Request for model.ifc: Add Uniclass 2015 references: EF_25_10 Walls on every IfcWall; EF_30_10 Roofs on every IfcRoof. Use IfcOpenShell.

First a look at what the model holds.

```python
import ifcopenshell

model = ifcopenshell.open("model.ifc")
print(model.schema)
print("classifications:", [c.Name for c in model.by_type("IfcClassification")])
for ifc_class in ("IfcDoor", "IfcRoof", "IfcStair", "IfcWall", "IfcWindow"):
    print(ifc_class, len(model.by_type(ifc_class)))
```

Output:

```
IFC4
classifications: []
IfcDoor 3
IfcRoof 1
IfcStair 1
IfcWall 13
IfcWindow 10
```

```python
import ifcopenshell
import ifcopenshell.api.classification

model = ifcopenshell.open("model.ifc")

system = ifcopenshell.api.classification.add_classification(model, classification="Uniclass 2015")

codes = {
    "IfcWall": ("EF_25_10", "Walls"),
    "IfcRoof": ("EF_30_10", "Roofs"),
}
for ifc_class, (code, name) in codes.items():
    products = model.by_type(ifc_class)
    ifcopenshell.api.classification.add_reference(
        model, products=products, classification=system, identification=code, name=name
    )
    print(code, len(products))

model.write("model_updated.ifc")
```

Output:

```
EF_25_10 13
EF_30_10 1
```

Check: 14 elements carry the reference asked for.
